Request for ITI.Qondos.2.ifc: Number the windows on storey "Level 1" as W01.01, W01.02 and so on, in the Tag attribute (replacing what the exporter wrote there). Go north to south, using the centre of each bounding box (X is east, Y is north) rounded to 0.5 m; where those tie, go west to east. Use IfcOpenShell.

First a look at what the model holds.

```python
import ifcopenshell
import ifcopenshell.util.element
import ifcopenshell.util.placement

model = ifcopenshell.open("ITI.Qondos.2.ifc")
print(model.schema)
storey = next(s for s in model.by_type("IfcBuildingStorey") if s.Name == "Level 1")
windows = [e for e in ifcopenshell.util.element.get_decomposition(storey) if e.is_a("IfcWindow")]
for e in sorted(windows, key=lambda e: e.id()):
    origin = ifcopenshell.util.placement.get_local_placement(e.ObjectPlacement)[:3, 3]
    print(e.id(), e.Tag, e.Name, origin.round(2) + 0.0, sep=" | ")
```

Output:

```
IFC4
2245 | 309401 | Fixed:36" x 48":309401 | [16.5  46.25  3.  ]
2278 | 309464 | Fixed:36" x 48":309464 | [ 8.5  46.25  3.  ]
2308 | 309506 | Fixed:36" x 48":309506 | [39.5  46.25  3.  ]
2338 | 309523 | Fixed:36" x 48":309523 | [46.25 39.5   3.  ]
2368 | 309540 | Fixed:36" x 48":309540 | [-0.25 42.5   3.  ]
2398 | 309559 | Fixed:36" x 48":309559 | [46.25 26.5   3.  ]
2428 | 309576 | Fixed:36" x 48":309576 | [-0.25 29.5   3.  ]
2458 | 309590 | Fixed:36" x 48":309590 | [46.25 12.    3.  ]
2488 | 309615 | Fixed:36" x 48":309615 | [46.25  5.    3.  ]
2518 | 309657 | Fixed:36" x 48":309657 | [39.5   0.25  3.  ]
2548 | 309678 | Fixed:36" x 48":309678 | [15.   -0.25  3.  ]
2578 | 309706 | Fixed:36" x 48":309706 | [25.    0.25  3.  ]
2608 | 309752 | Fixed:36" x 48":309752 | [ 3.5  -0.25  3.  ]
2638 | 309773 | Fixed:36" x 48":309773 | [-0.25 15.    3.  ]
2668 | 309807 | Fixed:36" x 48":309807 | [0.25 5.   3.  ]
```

```python
import ifcopenshell
import ifcopenshell.geom
import ifcopenshell.util.element
import ifcopenshell.util.shape

model = ifcopenshell.open("ITI.Qondos.2.ifc")
settings = ifcopenshell.geom.settings()
settings.set("use-world-coords", True)


def centre(element):
    shape = ifcopenshell.geom.create_shape(settings, element)
    return ifcopenshell.util.shape.get_bbox_centroid(shape.geometry)


storey = next(s for s in model.by_type("IfcBuildingStorey") if s.Name == "Level 1")
windows = [e for e in ifcopenshell.util.element.get_decomposition(storey) if e.is_a("IfcWindow")]

# Insertion points can sit at a corner or the storey origin, so sort by the geometry (in metres).
centres = {e: centre(e) for e in windows}
windows.sort(key=lambda e: (-round(centres[e][1] / 0.5), centres[e][0]))

for i, e in enumerate(windows, start=1):
    number = f"W01.{i:02d}"
    e.Tag = number
    print(e.id(), number)

model.write("ITI.Qondos.2_edited.ifc")
```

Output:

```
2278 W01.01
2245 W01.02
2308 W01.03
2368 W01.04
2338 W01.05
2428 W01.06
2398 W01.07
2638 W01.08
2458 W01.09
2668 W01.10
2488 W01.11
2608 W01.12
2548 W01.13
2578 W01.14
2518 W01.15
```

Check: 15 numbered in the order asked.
